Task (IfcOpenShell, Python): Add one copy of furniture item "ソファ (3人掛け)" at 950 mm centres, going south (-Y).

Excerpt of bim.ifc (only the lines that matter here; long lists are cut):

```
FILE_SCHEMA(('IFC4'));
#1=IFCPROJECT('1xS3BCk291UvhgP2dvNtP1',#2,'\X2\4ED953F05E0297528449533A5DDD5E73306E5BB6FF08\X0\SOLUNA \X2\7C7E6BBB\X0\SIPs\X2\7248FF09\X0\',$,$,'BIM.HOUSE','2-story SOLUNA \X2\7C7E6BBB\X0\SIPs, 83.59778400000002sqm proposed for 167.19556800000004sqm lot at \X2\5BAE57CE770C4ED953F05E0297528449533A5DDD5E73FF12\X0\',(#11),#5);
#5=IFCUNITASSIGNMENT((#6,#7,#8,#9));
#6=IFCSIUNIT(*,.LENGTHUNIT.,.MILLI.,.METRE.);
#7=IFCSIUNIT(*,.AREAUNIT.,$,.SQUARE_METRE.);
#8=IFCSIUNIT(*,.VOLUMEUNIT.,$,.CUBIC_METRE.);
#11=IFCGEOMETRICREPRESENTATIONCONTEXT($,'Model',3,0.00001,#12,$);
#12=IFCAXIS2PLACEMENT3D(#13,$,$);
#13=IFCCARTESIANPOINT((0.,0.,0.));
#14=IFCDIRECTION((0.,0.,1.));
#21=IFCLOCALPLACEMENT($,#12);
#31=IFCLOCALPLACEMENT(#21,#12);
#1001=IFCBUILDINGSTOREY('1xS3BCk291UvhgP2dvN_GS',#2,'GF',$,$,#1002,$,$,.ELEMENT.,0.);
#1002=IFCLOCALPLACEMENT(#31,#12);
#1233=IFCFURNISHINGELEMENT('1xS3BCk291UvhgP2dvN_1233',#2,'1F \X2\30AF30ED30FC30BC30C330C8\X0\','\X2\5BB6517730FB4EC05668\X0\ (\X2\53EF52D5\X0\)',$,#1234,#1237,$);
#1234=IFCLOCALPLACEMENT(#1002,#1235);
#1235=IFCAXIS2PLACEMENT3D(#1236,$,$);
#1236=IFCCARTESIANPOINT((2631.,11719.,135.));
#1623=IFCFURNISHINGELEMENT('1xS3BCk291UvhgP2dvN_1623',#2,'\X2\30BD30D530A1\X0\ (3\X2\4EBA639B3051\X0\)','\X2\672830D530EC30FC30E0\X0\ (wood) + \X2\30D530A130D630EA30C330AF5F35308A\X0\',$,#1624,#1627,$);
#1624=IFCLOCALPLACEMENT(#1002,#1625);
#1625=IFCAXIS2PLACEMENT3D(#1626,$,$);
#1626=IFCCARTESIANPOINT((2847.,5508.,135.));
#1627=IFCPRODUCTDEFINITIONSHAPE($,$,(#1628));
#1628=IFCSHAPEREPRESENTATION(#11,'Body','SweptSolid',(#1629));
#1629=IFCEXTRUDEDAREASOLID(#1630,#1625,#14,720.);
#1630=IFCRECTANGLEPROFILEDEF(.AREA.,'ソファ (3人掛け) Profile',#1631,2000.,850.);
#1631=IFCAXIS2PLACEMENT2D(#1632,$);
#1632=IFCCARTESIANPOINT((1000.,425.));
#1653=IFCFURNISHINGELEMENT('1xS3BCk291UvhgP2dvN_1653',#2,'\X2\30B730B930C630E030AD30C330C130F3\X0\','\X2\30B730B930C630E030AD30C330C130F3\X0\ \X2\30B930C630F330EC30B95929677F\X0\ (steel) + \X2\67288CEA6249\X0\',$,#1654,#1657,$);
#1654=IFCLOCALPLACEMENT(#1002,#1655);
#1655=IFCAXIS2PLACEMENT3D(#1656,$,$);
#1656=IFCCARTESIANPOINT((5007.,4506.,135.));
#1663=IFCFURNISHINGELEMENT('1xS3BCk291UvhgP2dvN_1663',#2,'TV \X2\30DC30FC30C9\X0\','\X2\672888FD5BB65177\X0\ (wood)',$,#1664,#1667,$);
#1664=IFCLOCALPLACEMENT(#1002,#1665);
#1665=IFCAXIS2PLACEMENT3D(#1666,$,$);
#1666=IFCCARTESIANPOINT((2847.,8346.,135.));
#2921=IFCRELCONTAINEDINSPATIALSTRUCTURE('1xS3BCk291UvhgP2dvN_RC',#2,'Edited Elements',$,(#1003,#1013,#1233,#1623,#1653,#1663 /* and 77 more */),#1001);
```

```python
import numpy as np
import ifcopenshell
import ifcopenshell.api.geometry
import ifcopenshell.api.root
import ifcopenshell.util.element
import ifcopenshell.util.placement

model = ifcopenshell.open("bim.ifc")


def reuse_history(source, copy):
    """copy_class also copies each property set's owner history, people and application; keep the originals."""
    for rel in copy.IsDefinedBy:
        if rel.is_a("IfcRelDefinesByProperties") and (history := rel.RelatingPropertyDefinition.OwnerHistory):
            rel.RelatingPropertyDefinition.OwnerHistory = source.OwnerHistory
            ifcopenshell.util.element.remove_deep2(model, history)


source = model.by_id(1623)
base = ifcopenshell.util.placement.get_local_placement(source.ObjectPlacement)
step = np.array([0.0, -1.0, 0.0]) * 950.0

for i in range(1, 2):
    copy = ifcopenshell.api.root.copy_class(model, product=source)
    copy.Representation = ifcopenshell.util.element.copy_deep(
        model, source.Representation, exclude=["IfcGeometricRepresentationContext", "IfcRepresentationMap"]
    )
    reuse_history(source, copy)
    matrix = base.copy()
    matrix[:3, 3] += i * step
    print("added at", matrix[:3, 3].round(3) + 0.0)
    ifcopenshell.api.geometry.edit_object_placement(model, product=copy, matrix=matrix, is_si=False)

model.write("bim_edited.ifc")
```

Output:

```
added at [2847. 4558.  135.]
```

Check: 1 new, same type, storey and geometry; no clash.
